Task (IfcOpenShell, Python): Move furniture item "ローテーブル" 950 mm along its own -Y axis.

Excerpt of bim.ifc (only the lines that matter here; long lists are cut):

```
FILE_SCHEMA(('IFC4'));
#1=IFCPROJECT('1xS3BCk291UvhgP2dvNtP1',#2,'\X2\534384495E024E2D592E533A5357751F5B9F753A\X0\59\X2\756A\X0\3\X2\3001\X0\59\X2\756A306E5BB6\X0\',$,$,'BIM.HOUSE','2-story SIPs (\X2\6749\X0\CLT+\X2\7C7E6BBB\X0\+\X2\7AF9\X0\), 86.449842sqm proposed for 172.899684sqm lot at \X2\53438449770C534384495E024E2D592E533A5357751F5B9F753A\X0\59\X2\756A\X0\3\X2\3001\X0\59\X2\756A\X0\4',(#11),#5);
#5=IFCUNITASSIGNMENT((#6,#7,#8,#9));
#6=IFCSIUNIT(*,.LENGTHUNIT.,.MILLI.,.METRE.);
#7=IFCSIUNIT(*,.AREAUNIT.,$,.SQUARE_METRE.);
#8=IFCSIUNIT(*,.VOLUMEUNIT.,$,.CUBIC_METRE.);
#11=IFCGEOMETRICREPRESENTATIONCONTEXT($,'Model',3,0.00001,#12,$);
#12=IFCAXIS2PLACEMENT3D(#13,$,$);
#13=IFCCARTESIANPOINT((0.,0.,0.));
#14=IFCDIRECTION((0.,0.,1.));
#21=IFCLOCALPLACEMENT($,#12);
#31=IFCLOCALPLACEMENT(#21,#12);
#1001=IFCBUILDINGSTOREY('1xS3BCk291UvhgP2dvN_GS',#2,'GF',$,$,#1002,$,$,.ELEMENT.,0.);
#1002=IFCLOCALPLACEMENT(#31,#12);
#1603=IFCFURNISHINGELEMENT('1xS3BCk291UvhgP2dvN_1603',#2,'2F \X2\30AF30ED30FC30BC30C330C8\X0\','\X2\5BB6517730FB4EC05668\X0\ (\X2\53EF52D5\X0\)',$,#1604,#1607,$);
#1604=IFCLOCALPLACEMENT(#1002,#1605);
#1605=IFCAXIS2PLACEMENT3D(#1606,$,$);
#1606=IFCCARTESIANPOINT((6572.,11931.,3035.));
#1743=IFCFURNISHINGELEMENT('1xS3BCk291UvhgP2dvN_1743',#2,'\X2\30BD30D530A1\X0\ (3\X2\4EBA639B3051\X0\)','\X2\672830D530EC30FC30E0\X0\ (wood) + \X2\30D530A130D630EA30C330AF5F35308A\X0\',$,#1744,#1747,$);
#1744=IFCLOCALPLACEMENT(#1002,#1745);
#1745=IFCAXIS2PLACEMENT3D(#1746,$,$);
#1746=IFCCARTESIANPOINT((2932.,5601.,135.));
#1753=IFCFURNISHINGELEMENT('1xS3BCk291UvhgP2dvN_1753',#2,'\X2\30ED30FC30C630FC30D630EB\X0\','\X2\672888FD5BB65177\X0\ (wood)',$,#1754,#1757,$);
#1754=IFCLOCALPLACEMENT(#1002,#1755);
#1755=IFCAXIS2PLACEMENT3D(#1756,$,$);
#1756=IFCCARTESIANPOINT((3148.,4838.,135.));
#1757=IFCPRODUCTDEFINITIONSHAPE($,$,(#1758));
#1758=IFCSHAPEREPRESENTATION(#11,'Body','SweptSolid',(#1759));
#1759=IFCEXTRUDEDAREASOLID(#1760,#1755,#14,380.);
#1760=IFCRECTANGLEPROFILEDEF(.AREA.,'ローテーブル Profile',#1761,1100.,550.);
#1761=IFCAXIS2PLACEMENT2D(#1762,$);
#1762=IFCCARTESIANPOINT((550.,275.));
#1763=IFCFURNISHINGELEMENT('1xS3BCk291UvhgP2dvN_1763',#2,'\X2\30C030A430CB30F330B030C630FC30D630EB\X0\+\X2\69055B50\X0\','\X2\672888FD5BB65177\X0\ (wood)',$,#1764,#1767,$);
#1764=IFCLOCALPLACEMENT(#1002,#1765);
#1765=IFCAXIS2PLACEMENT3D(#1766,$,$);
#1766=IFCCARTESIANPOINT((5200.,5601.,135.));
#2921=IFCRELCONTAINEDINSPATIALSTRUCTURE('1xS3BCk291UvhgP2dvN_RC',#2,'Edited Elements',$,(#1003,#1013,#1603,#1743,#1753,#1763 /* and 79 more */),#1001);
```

```python
import ifcopenshell
import ifcopenshell.api.geometry
import ifcopenshell.util.placement

model = ifcopenshell.open("bim.ifc")

item = model.by_id(1753)
matrix = ifcopenshell.util.placement.get_local_placement(item.ObjectPlacement)
matrix[:3, 3] -= matrix[:3, 1] * 950.0
ifcopenshell.api.geometry.edit_object_placement(model, product=item, matrix=matrix, is_si=False)

print(ifcopenshell.util.placement.get_local_placement(item.ObjectPlacement).round(3) + 0.0)

model.write("bim_rev.ifc")
```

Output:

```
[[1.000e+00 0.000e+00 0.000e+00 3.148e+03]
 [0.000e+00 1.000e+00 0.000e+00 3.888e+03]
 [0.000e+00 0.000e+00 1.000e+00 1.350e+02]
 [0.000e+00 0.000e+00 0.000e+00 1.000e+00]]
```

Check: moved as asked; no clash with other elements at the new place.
